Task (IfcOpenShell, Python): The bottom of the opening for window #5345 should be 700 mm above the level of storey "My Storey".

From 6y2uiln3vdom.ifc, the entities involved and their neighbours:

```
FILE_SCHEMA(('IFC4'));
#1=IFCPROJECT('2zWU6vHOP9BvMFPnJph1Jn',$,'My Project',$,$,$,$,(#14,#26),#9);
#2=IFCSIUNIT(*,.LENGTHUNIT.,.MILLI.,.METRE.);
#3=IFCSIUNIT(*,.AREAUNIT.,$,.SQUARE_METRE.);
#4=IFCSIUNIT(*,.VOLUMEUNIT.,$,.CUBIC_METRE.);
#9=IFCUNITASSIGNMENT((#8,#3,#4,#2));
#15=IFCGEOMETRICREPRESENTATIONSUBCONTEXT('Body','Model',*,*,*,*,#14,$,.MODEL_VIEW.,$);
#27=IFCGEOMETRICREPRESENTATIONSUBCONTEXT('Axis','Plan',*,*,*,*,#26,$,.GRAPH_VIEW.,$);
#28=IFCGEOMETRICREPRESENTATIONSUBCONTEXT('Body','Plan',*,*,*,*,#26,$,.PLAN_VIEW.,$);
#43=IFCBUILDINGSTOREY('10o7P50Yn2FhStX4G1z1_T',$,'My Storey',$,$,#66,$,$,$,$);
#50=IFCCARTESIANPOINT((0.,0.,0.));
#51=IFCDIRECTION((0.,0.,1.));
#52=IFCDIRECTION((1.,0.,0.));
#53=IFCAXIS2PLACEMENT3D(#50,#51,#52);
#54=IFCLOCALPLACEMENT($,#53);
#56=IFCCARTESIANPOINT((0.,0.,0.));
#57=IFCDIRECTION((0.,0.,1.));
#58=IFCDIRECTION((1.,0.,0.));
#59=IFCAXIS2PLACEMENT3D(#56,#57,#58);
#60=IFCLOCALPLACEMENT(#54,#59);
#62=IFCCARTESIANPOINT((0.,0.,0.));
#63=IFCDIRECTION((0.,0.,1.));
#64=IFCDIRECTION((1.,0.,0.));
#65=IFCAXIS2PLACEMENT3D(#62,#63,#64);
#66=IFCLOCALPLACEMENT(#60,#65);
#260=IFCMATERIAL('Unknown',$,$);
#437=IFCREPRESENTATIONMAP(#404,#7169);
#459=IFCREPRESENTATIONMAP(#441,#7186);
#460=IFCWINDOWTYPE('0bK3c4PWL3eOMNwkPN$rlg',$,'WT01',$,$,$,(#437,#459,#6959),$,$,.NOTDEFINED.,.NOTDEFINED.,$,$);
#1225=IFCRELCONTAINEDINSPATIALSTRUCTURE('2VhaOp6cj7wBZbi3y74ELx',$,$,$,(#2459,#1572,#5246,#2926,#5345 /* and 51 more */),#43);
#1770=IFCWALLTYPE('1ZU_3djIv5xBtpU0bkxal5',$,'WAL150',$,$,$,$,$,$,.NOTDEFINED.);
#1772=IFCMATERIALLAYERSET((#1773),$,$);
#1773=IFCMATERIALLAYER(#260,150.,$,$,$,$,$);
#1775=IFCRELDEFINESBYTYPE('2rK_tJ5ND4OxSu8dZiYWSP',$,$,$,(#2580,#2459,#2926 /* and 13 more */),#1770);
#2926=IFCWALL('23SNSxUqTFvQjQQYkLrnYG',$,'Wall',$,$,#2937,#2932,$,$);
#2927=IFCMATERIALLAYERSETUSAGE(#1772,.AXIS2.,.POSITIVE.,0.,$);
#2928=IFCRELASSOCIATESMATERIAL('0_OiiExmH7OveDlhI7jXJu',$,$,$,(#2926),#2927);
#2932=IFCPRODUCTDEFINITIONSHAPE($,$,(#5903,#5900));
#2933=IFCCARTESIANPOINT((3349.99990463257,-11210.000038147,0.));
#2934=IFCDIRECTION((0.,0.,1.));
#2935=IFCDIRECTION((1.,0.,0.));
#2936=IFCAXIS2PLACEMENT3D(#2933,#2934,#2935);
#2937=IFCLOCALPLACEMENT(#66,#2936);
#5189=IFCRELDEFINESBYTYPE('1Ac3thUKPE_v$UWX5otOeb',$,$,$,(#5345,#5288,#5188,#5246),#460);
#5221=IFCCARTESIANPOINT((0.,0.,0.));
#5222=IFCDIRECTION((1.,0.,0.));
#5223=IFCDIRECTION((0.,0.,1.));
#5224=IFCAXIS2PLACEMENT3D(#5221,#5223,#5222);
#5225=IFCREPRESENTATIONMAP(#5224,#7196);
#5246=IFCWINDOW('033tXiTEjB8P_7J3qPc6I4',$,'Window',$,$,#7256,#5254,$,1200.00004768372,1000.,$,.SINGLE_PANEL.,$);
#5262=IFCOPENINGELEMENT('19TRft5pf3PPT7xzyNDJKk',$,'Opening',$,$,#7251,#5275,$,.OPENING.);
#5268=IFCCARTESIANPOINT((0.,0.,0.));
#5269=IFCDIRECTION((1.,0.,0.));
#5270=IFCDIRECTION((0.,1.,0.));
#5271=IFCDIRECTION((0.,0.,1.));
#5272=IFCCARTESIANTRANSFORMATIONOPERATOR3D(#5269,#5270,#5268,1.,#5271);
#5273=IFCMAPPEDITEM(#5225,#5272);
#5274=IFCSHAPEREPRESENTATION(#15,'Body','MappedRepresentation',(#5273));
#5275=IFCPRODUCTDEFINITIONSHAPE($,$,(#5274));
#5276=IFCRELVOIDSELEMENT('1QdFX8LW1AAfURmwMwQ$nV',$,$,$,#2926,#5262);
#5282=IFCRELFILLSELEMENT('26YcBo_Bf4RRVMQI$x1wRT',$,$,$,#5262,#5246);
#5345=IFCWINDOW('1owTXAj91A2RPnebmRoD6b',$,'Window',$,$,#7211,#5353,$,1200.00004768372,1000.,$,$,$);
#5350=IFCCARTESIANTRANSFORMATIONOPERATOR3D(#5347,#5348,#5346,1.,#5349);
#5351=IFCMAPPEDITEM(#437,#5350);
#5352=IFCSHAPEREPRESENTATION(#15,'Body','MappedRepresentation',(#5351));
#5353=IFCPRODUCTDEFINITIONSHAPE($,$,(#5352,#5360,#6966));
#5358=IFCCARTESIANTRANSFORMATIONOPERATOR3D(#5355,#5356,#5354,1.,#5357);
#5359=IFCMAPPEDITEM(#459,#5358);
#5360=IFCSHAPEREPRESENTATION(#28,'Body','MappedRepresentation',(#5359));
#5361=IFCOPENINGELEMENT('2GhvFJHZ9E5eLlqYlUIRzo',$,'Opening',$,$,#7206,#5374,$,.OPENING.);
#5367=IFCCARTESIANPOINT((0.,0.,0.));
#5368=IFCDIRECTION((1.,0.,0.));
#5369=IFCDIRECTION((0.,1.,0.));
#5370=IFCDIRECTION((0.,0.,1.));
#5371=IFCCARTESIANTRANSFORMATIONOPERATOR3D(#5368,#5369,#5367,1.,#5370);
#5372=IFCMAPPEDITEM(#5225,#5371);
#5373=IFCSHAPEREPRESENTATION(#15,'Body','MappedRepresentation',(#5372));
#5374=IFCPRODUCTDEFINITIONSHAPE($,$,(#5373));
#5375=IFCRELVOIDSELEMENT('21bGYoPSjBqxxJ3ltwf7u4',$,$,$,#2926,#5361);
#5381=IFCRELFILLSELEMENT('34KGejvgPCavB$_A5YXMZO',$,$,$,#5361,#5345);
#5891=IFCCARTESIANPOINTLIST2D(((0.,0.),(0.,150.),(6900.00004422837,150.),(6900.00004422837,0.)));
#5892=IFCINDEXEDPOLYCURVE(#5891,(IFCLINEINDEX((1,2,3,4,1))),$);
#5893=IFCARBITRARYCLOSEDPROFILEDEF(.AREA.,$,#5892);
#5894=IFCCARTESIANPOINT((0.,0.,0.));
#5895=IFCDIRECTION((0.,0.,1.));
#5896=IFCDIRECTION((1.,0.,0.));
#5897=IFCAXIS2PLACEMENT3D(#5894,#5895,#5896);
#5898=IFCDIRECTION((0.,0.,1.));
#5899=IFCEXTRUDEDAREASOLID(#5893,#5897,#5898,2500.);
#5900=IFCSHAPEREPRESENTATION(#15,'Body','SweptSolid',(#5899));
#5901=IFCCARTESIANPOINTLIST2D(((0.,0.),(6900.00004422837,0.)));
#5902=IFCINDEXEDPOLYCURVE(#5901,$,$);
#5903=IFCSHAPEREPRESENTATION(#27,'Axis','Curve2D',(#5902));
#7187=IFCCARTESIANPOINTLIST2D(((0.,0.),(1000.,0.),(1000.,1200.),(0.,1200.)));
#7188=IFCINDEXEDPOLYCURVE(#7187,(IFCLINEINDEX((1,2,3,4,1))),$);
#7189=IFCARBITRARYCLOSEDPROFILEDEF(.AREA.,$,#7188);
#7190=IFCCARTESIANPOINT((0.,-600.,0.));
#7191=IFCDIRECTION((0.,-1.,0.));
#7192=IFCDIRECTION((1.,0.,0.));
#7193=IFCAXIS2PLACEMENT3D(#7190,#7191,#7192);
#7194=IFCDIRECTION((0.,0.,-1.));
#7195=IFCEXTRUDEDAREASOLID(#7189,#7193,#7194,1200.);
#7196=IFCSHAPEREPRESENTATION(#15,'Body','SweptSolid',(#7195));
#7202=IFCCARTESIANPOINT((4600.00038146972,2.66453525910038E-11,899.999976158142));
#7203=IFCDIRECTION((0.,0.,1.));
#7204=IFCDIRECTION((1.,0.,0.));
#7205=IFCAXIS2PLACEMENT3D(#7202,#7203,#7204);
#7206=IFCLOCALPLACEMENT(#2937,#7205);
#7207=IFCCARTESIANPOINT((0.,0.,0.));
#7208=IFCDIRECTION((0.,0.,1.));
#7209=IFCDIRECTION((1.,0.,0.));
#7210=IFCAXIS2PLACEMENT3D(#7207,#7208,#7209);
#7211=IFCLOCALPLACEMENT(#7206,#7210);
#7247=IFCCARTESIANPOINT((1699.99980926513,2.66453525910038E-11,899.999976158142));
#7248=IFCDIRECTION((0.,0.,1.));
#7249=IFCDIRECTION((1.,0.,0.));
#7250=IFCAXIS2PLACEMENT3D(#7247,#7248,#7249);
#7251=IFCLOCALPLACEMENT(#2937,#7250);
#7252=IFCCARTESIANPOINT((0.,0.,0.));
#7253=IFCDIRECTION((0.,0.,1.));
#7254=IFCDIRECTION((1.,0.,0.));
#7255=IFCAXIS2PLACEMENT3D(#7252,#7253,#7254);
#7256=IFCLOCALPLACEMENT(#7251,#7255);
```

```python
import numpy as np
import ifcopenshell
import ifcopenshell.api.geometry
import ifcopenshell.geom
import ifcopenshell.util.element
import ifcopenshell.util.placement
import ifcopenshell.util.shape
import ifcopenshell.util.unit

model = ifcopenshell.open("6y2uiln3vdom.ifc")
unit_scale = ifcopenshell.util.unit.calculate_unit_scale(model)

window = model.by_id(5345)
opening = window.FillsVoids[0].RelatingOpeningElement
storey = ifcopenshell.util.element.get_container(window, ifc_class="IfcBuildingStorey")
level = ifcopenshell.util.placement.get_local_placement(storey.ObjectPlacement)[2, 3]

# The opening's origin need not be at the sill, so measure its lowest point.
shape = ifcopenshell.geom.create_shape(ifcopenshell.geom.settings(), opening)
bottom = ifcopenshell.util.shape.get_shape_bottom_elevation(shape, shape.geometry) / unit_scale
dz = level + 0.7 / unit_scale - bottom

shift = np.array([0.0, 0.0, dz])
# The window is placed relative to its opening, so it follows when the opening moves.
matrix = ifcopenshell.util.placement.get_local_placement(opening.ObjectPlacement)
matrix[:3, 3] += shift
ifcopenshell.api.geometry.edit_object_placement(
    model, product=opening, matrix=matrix, is_si=False, should_transform_children=True
)

print(f"moved by {dz * unit_scale:+.3f} m")

model.write("6y2uiln3vdom_v2.ifc")
```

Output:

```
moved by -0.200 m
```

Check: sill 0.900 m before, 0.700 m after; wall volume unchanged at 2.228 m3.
